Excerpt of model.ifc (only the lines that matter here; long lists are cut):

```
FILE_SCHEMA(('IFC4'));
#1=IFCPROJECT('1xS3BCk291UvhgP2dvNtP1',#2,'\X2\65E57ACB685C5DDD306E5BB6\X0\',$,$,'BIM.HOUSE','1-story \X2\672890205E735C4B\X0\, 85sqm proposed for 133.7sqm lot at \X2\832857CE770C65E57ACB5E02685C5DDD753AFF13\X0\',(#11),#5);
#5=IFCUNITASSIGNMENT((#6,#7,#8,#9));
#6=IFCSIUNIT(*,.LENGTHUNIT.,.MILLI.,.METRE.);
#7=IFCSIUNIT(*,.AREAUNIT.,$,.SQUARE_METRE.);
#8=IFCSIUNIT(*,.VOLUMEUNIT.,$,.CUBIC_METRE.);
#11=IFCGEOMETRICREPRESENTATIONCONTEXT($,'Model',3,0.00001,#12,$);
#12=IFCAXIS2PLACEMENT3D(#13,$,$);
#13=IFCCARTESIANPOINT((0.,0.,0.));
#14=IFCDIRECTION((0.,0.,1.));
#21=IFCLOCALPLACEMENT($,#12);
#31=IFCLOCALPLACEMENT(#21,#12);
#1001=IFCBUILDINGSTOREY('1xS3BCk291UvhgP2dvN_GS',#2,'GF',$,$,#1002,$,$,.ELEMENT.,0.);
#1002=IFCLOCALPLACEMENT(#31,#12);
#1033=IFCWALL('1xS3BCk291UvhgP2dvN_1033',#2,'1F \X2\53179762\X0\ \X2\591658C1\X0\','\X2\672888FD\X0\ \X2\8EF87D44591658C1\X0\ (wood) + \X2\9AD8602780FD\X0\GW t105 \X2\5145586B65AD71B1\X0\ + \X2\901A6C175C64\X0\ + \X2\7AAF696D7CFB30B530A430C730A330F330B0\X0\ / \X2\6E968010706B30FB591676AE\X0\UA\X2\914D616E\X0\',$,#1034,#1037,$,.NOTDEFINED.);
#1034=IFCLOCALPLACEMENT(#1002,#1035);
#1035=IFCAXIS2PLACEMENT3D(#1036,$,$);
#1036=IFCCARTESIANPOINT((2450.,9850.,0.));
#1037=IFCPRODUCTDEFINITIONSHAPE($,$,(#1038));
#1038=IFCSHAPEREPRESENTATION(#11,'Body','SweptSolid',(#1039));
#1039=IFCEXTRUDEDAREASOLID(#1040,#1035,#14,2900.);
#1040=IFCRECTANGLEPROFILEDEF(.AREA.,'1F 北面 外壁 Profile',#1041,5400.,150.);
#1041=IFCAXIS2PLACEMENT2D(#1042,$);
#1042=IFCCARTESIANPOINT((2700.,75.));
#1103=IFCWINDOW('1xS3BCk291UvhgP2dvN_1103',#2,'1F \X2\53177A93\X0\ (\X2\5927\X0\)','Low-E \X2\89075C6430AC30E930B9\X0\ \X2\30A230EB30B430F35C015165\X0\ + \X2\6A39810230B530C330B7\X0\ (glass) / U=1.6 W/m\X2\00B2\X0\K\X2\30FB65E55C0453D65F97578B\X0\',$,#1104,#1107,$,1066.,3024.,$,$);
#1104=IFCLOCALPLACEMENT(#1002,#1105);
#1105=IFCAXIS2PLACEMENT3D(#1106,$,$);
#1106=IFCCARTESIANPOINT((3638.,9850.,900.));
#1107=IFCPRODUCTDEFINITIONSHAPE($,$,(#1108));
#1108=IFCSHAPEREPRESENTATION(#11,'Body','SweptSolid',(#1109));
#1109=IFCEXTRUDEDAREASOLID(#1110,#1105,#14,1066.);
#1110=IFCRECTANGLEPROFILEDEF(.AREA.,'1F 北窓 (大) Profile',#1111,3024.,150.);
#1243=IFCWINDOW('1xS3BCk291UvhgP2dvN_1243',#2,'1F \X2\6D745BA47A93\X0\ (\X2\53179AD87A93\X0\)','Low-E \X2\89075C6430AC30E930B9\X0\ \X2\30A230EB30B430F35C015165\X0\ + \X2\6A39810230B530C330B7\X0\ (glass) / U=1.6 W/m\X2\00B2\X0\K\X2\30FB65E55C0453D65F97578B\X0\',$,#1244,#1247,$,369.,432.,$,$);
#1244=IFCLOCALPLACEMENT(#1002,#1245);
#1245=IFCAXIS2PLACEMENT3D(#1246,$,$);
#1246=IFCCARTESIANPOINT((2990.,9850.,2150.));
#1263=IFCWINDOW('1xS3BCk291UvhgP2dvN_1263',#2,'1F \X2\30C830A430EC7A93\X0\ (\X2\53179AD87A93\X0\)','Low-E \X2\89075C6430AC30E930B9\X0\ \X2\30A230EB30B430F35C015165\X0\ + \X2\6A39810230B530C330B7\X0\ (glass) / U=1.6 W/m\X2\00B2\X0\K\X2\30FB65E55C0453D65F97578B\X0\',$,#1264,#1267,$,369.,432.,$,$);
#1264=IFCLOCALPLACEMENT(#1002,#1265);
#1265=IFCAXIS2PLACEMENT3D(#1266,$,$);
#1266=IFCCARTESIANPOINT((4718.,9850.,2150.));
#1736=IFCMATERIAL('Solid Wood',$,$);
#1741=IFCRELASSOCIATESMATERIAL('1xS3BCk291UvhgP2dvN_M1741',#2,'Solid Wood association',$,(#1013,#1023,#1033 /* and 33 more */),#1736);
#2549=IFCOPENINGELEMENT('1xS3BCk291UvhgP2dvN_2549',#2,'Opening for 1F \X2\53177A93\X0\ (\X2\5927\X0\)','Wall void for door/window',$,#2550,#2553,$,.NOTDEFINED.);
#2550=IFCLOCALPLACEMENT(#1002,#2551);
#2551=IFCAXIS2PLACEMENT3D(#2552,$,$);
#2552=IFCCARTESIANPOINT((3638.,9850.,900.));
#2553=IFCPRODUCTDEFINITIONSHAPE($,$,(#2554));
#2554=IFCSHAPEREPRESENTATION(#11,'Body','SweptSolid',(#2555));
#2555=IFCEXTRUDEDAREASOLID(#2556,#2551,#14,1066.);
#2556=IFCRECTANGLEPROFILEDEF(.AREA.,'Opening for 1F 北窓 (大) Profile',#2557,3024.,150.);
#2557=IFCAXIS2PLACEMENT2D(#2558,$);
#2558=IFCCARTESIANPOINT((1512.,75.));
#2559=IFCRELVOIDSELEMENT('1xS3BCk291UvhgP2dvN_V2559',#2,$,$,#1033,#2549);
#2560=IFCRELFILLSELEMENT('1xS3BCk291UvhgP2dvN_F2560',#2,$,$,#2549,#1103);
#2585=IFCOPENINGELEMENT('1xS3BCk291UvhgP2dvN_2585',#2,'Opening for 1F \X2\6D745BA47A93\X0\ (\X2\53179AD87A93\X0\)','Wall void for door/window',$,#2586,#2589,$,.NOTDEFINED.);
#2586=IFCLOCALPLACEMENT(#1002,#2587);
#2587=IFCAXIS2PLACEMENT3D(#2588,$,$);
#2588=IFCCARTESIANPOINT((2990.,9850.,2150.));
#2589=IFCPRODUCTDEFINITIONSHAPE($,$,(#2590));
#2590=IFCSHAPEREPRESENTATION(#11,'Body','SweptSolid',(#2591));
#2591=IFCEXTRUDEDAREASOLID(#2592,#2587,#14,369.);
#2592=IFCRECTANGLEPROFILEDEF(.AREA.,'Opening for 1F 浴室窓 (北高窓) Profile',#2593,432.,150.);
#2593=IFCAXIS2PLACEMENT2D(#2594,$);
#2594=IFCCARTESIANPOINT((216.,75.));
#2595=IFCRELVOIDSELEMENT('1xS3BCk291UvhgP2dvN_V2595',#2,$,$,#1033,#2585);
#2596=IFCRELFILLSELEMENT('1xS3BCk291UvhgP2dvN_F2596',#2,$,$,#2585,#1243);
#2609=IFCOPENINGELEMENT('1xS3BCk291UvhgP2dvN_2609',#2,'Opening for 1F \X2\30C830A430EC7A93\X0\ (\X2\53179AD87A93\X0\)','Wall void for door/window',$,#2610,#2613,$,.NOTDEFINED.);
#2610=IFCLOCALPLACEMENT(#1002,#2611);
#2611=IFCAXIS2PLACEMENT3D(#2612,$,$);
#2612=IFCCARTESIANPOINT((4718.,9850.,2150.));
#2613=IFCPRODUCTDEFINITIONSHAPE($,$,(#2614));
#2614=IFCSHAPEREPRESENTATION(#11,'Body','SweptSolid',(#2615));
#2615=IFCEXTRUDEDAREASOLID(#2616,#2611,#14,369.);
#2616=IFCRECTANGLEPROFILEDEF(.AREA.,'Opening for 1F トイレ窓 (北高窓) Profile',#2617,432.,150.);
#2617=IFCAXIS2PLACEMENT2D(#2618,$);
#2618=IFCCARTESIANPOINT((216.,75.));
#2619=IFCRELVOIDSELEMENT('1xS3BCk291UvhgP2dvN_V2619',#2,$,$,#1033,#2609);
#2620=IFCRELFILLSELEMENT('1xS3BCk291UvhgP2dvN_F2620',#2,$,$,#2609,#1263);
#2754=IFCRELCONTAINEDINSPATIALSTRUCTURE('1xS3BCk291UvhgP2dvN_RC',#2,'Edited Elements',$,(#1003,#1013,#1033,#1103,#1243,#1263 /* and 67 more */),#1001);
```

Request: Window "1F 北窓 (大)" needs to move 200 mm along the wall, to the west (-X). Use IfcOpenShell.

```python
import ifcopenshell
import ifcopenshell.api.geometry
import ifcopenshell.util.placement
import ifcopenshell.util.unit

model = ifcopenshell.open("model.ifc")
unit_scale = ifcopenshell.util.unit.calculate_unit_scale(model)

window = model.by_id(1103)
opening = window.FillsVoids[0].RelatingOpeningElement
wall = opening.VoidsElements[0].RelatingBuildingElement

wall_matrix = ifcopenshell.util.placement.get_local_placement(wall.ObjectPlacement)
shift = wall_matrix[:3, 0] * -0.2 / unit_scale
before = ifcopenshell.util.placement.get_local_placement(window.ObjectPlacement)[:3, 3].copy()

# The window is not placed relative to its opening, so move both.
for product in (opening, window):
    matrix = ifcopenshell.util.placement.get_local_placement(product.ObjectPlacement)
    matrix[:3, 3] += shift
    ifcopenshell.api.geometry.edit_object_placement(model, product=product, matrix=matrix, is_si=False)

after = ifcopenshell.util.placement.get_local_placement(window.ObjectPlacement)[:3, 3]
print("window moved by", (after - before).round(3) + 0.0)

model.write("model_updated.ifc")
```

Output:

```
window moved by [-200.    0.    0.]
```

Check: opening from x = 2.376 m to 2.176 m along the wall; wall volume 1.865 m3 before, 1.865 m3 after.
